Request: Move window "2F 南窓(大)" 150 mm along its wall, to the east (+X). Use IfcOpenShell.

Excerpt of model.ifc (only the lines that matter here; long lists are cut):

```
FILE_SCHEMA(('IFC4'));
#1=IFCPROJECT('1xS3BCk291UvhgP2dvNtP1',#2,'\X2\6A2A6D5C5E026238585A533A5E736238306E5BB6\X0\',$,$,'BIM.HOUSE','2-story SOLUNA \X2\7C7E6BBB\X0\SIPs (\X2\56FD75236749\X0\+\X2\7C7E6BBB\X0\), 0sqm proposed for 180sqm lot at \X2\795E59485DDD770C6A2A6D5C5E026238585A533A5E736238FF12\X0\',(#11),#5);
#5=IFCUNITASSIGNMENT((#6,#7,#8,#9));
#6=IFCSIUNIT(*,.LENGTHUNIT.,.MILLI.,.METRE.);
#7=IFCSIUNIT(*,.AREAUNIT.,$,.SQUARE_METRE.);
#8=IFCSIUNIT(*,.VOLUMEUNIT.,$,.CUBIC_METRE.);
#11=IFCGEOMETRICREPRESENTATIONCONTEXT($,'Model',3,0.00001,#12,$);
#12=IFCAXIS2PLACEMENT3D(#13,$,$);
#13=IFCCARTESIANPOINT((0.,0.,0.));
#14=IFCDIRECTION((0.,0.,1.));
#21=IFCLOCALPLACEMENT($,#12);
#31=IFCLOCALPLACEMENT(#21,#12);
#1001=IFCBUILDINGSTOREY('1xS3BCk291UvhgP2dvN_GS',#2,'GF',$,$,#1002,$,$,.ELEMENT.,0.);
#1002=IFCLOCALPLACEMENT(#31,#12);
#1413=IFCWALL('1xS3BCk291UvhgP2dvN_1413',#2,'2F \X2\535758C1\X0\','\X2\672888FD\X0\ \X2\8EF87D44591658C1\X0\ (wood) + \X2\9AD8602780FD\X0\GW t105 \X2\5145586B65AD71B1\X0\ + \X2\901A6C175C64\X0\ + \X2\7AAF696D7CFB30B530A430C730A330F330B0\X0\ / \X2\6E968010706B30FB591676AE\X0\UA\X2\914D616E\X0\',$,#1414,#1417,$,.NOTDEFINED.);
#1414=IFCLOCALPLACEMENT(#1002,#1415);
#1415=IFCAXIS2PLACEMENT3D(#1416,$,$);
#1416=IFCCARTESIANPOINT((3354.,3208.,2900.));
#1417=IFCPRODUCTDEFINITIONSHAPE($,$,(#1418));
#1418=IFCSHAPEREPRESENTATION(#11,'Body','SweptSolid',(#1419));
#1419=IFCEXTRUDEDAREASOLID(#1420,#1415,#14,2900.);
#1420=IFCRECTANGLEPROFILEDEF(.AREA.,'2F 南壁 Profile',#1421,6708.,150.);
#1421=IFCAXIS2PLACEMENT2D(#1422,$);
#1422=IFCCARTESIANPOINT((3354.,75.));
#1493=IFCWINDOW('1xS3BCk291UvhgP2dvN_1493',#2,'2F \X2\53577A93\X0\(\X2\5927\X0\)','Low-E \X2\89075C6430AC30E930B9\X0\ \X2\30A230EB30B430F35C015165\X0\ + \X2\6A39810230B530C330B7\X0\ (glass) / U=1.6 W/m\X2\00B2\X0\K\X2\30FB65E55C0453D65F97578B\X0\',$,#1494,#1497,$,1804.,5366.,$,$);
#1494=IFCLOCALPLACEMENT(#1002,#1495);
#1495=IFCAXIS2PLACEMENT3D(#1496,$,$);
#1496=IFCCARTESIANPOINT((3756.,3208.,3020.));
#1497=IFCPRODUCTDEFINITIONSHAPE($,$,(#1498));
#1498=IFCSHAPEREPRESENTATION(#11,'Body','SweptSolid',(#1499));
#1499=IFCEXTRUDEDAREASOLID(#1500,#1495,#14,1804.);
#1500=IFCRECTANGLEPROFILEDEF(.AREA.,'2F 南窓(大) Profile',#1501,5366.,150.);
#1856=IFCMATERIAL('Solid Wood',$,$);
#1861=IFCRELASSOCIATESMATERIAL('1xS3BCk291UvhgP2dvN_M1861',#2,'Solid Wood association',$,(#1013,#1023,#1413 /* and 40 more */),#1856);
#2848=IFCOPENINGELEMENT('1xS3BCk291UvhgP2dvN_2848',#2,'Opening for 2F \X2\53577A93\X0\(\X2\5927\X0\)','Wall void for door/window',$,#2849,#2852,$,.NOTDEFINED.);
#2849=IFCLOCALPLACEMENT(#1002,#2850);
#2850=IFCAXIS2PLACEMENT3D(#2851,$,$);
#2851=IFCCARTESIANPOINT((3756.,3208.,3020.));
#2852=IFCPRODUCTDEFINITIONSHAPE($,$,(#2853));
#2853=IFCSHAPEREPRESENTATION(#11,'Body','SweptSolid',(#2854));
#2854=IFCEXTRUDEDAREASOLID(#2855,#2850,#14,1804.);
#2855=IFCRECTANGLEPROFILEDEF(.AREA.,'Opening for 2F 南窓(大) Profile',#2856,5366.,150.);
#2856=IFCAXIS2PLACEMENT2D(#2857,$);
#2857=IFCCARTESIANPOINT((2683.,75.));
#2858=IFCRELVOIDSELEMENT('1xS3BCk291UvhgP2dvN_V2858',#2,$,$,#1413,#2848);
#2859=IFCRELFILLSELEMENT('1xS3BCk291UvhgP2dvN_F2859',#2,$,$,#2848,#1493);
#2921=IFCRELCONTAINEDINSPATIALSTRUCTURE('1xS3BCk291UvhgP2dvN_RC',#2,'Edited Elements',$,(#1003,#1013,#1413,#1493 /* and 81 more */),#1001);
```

```python
import ifcopenshell
import ifcopenshell.api.geometry
import ifcopenshell.util.placement
import ifcopenshell.util.unit

model = ifcopenshell.open("model.ifc")
unit_scale = ifcopenshell.util.unit.calculate_unit_scale(model)

window = model.by_guid("1xS3BCk291UvhgP2dvN_1493")
opening = window.FillsVoids[0].RelatingOpeningElement
wall = opening.VoidsElements[0].RelatingBuildingElement

wall_matrix = ifcopenshell.util.placement.get_local_placement(wall.ObjectPlacement)
shift = wall_matrix[:3, 0] * 0.15 / unit_scale
before = ifcopenshell.util.placement.get_local_placement(window.ObjectPlacement)[:3, 3].copy()

# The window is not placed relative to its opening, so move both.
for product in (opening, window):
    matrix = ifcopenshell.util.placement.get_local_placement(product.ObjectPlacement)
    matrix[:3, 3] += shift
    ifcopenshell.api.geometry.edit_object_placement(model, product=product, matrix=matrix, is_si=False)

after = ifcopenshell.util.placement.get_local_placement(window.ObjectPlacement)[:3, 3]
print("window moved by", (after - before).round(3) + 0.0)

model.write("model_rev.ifc")
```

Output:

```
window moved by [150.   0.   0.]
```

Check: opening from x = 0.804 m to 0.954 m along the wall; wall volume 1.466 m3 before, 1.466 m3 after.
